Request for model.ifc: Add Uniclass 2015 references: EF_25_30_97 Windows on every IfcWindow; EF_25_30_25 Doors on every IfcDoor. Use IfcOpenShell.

First a look at what the model holds.

```python
import ifcopenshell

model = ifcopenshell.open("model.ifc")
print(model.schema)
print("classifications:", [c.Name for c in model.by_type("IfcClassification")])
for ifc_class in ("IfcDoor", "IfcRoof", "IfcStair", "IfcWall", "IfcWindow"):
    print(ifc_class, len(model.by_type(ifc_class)))
```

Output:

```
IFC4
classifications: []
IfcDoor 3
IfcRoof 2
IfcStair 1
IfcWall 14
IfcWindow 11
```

```python
import ifcopenshell
import ifcopenshell.api.classification

model = ifcopenshell.open("model.ifc")

system = ifcopenshell.api.classification.add_classification(model, classification="Uniclass 2015")

codes = {
    "IfcWindow": ("EF_25_30_97", "Windows"),
    "IfcDoor": ("EF_25_30_25", "Doors"),
}
for ifc_class, (code, name) in codes.items():
    products = model.by_type(ifc_class)
    ifcopenshell.api.classification.add_reference(
        model, products=products, classification=system, identification=code, name=name
    )
    print(code, len(products))

model.write("model_edited.ifc")
```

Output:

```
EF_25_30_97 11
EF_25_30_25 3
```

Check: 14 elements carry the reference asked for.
